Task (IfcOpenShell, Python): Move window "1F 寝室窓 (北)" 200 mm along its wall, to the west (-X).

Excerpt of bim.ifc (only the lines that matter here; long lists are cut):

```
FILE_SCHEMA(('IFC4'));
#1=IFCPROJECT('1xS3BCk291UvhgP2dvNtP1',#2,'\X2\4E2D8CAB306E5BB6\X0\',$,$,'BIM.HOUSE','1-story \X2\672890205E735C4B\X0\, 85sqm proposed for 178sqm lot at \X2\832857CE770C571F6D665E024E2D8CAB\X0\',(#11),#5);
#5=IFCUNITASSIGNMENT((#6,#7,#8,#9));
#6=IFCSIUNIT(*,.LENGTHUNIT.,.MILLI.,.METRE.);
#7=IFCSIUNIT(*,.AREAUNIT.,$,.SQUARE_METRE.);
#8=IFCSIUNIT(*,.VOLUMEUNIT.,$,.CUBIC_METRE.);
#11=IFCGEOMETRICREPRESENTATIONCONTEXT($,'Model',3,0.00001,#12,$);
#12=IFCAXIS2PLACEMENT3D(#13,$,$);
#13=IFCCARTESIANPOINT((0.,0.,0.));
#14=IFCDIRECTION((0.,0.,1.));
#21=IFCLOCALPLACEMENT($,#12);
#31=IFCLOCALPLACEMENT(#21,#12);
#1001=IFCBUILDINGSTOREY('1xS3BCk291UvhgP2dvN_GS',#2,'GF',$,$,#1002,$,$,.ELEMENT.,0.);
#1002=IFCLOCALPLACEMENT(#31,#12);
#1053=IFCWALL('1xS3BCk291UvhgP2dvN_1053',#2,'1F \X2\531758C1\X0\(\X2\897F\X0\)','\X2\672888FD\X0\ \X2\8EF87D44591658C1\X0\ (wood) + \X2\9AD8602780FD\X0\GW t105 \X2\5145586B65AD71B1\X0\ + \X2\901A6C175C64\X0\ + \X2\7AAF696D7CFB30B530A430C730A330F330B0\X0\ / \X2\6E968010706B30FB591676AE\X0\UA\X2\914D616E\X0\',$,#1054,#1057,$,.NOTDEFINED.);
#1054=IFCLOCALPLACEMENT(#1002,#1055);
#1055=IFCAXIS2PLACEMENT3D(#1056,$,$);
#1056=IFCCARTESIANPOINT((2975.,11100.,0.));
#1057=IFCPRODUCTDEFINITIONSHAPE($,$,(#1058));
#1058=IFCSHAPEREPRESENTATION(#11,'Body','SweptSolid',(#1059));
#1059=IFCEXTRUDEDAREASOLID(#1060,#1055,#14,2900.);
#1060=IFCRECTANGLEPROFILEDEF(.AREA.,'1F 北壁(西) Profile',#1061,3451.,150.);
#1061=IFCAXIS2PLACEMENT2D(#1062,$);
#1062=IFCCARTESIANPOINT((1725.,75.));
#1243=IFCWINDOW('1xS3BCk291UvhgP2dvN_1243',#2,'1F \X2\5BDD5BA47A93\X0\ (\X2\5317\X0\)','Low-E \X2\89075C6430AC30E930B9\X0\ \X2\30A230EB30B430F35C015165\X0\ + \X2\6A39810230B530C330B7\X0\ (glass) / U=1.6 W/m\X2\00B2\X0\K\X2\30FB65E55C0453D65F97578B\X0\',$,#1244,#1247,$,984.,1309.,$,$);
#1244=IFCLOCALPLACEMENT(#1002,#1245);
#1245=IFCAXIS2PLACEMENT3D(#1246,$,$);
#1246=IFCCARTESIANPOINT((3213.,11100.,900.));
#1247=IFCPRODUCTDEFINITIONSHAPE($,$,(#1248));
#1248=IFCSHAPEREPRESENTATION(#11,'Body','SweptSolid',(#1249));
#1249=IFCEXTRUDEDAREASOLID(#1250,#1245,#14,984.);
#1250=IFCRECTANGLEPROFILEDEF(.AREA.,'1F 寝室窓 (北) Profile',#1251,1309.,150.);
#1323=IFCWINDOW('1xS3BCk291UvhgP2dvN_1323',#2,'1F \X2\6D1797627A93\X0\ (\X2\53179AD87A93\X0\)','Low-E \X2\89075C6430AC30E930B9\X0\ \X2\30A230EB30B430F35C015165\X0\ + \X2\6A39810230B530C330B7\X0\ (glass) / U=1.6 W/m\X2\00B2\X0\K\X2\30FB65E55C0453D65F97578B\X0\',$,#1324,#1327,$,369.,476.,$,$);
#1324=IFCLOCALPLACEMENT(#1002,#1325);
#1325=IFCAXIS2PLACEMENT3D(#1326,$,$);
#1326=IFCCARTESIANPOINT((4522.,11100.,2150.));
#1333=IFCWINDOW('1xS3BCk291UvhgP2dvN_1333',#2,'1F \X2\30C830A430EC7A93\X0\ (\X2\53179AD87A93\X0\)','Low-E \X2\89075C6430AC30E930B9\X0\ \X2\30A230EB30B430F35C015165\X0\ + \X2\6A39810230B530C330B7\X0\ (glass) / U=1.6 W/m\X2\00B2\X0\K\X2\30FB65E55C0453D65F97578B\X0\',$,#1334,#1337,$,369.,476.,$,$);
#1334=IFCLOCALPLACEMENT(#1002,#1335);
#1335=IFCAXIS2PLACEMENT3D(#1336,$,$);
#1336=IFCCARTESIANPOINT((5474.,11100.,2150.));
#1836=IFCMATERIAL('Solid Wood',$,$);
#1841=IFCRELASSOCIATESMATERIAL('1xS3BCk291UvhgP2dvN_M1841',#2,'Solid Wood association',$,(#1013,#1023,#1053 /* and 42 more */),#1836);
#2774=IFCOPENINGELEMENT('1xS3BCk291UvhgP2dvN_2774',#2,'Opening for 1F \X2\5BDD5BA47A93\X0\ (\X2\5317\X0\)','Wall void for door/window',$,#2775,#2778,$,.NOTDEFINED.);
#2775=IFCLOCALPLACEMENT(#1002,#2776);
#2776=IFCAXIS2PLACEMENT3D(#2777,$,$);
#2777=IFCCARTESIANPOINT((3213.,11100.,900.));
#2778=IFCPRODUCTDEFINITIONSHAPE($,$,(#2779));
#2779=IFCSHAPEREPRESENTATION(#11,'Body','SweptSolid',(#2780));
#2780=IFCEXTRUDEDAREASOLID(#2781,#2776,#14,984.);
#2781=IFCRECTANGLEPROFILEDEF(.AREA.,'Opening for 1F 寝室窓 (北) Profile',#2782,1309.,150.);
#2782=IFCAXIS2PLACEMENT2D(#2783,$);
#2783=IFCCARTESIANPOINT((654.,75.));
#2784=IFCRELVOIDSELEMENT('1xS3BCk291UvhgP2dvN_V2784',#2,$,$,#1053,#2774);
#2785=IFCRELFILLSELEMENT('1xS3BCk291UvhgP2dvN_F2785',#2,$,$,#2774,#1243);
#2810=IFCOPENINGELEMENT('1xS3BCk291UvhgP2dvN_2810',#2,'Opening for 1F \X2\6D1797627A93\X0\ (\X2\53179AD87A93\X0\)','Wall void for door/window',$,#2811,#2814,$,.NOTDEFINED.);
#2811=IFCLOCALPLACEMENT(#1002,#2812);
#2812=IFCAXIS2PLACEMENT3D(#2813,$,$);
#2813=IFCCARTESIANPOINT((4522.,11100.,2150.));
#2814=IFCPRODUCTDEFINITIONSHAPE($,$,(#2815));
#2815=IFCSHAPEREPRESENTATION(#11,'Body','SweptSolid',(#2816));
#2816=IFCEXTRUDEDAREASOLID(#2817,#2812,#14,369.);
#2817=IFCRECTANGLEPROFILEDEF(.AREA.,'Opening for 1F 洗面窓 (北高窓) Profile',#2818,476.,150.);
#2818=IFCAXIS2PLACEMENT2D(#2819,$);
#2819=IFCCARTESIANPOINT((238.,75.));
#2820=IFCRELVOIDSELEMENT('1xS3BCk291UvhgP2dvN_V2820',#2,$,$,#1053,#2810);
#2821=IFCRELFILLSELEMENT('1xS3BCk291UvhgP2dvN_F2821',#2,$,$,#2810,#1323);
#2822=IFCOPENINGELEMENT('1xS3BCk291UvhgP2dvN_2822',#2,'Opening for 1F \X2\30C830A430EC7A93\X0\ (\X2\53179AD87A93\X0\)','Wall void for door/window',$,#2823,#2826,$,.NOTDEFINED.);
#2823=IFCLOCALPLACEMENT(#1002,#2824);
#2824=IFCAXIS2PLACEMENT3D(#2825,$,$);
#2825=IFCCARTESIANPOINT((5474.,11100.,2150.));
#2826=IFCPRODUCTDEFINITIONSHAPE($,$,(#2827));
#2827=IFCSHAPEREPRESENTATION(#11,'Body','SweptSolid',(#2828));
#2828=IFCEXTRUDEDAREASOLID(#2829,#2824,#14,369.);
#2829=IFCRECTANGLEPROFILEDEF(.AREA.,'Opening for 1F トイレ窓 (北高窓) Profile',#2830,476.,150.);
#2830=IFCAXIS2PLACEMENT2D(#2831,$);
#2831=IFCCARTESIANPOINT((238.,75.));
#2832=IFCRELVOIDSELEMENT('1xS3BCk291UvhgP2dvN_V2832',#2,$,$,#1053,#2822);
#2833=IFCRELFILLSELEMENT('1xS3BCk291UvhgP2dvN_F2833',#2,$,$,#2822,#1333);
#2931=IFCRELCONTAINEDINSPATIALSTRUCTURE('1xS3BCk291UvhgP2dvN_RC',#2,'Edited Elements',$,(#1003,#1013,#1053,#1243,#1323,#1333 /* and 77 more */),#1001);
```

```python
import ifcopenshell
import ifcopenshell.api.geometry
import ifcopenshell.util.placement

model = ifcopenshell.open("bim.ifc")

window = model.by_id(1243)
opening = window.FillsVoids[0].RelatingOpeningElement
wall = opening.VoidsElements[0].RelatingBuildingElement

wall_matrix = ifcopenshell.util.placement.get_local_placement(wall.ObjectPlacement)
shift = wall_matrix[:3, 0] * -200.0
before = ifcopenshell.util.placement.get_local_placement(window.ObjectPlacement)[:3, 3].copy()

# The window is not placed relative to its opening, so move both.
for product in (opening, window):
    matrix = ifcopenshell.util.placement.get_local_placement(product.ObjectPlacement)
    matrix[:3, 3] += shift
    ifcopenshell.api.geometry.edit_object_placement(model, product=product, matrix=matrix, is_si=False)

after = ifcopenshell.util.placement.get_local_placement(window.ObjectPlacement)[:3, 3]
print("window moved by", (after - before).round(3) + 0.0)

model.write("bim_v2.ifc")
```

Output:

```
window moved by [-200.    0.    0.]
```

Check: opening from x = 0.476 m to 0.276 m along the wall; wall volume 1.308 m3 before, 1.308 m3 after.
